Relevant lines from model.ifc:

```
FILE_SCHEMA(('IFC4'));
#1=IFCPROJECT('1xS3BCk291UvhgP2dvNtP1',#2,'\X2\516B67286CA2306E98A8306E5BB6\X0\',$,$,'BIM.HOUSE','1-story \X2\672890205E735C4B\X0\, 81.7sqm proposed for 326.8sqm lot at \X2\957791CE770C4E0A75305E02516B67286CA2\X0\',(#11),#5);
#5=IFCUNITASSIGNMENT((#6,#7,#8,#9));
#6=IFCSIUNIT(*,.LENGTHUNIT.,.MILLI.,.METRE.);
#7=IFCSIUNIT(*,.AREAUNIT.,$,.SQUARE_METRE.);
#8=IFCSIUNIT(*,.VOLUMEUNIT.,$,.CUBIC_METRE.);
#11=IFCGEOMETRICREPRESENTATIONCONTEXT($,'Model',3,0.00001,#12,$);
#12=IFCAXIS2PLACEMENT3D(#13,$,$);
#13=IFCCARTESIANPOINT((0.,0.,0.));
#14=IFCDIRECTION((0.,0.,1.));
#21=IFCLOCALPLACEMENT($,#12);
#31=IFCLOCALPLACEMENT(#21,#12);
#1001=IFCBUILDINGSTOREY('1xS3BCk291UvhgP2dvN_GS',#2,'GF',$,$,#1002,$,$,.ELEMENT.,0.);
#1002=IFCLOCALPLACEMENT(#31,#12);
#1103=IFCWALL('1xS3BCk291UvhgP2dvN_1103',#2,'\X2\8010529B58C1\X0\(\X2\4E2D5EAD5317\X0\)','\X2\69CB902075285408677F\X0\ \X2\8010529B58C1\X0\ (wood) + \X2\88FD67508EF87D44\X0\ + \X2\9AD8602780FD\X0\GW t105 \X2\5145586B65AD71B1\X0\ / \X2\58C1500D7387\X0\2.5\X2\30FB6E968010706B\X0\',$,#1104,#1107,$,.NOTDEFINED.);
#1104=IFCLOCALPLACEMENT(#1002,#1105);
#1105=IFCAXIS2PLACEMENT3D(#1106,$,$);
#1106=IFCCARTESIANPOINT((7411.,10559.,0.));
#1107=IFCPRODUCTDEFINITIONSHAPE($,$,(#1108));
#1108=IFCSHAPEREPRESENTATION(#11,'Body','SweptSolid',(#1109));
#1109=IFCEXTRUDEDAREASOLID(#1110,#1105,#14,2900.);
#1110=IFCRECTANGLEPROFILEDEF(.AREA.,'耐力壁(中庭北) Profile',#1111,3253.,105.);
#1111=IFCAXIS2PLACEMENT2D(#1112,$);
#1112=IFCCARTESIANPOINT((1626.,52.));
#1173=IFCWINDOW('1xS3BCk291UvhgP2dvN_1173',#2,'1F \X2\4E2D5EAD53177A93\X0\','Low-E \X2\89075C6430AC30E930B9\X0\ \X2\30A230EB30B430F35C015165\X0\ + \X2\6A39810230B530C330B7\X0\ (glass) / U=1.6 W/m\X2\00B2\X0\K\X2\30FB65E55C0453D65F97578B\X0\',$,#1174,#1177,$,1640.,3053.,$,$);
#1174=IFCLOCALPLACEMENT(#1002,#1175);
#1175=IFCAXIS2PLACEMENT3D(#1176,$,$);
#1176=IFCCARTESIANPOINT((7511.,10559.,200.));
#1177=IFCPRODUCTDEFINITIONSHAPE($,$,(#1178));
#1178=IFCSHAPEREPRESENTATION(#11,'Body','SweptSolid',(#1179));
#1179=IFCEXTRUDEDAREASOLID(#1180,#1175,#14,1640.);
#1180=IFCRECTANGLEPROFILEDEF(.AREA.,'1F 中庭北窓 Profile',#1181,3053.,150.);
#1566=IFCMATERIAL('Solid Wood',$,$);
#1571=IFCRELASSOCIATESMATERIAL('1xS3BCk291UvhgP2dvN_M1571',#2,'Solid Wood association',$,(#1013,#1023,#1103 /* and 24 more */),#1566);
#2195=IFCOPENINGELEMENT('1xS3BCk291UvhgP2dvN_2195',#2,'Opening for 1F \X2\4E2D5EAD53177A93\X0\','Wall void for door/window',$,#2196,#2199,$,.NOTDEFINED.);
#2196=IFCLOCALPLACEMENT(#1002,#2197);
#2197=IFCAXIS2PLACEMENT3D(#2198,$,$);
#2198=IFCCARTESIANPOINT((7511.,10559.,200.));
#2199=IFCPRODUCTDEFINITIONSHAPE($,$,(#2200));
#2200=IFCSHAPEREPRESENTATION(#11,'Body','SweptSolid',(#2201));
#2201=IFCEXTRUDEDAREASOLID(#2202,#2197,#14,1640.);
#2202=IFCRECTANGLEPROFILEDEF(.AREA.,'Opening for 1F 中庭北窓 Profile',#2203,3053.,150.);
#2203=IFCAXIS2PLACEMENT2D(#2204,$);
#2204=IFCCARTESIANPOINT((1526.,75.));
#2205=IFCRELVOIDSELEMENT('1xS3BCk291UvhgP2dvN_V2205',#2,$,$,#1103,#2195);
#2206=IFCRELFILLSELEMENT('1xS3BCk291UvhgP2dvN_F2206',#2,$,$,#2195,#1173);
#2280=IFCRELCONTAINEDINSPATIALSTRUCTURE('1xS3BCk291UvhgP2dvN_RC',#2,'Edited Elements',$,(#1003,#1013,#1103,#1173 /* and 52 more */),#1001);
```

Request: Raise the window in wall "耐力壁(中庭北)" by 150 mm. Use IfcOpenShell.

```python
import numpy as np
import ifcopenshell
import ifcopenshell.api.geometry
import ifcopenshell.util.placement
import ifcopenshell.util.unit

model = ifcopenshell.open("model.ifc")
unit_scale = ifcopenshell.util.unit.calculate_unit_scale(model)

window = model.by_id(1173)
opening = window.FillsVoids[0].RelatingOpeningElement
dz = 150.0

shift = np.array([0.0, 0.0, dz])
# The window is not placed relative to its opening, so move both.
for product in (opening, window):
    matrix = ifcopenshell.util.placement.get_local_placement(product.ObjectPlacement)
    matrix[:3, 3] += shift
    ifcopenshell.api.geometry.edit_object_placement(model, product=product, matrix=matrix, is_si=False)

print(f"moved by {dz * unit_scale:+.3f} m")

model.write("model_v2.ifc")
```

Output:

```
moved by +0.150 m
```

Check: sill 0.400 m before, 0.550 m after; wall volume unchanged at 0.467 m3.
